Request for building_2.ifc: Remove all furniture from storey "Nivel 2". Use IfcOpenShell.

First a look at what the model holds.

```python
import ifcopenshell
import ifcopenshell.util.element

model = ifcopenshell.open("building_2.ifc")
print(model.schema)
storey = next(s for s in model.by_type("IfcBuildingStorey") if s.Name == "Nivel 2")
furniture = [e for e in ifcopenshell.util.element.get_decomposition(storey) if e.is_a("IfcFurnishingElement")]
seen = {}
for e in furniture:
    element_type = ifcopenshell.util.element.get_type(e)
    name = element_type.Name if element_type not in (None, e) else None
    seen[name] = seen.get(name, 0) + 1
for name, count in sorted(seen.items(), key=str):
    print(count, "x", name)
```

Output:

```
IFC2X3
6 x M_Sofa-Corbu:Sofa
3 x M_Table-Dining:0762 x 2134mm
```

```python
import ifcopenshell
import ifcopenshell.api.root
import ifcopenshell.util.element

model = ifcopenshell.open("building_2.ifc")

storey = next(s for s in model.by_type("IfcBuildingStorey") if s.Name == "Nivel 2")
furniture = [e for e in ifcopenshell.util.element.get_decomposition(storey) if e.is_a("IfcFurnishingElement")]

for e in furniture:
    ifcopenshell.api.root.remove_product(model, product=e)
print(len(furniture), "removed")

model.write("building_2-out.ifc")
```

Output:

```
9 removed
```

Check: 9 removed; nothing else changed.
